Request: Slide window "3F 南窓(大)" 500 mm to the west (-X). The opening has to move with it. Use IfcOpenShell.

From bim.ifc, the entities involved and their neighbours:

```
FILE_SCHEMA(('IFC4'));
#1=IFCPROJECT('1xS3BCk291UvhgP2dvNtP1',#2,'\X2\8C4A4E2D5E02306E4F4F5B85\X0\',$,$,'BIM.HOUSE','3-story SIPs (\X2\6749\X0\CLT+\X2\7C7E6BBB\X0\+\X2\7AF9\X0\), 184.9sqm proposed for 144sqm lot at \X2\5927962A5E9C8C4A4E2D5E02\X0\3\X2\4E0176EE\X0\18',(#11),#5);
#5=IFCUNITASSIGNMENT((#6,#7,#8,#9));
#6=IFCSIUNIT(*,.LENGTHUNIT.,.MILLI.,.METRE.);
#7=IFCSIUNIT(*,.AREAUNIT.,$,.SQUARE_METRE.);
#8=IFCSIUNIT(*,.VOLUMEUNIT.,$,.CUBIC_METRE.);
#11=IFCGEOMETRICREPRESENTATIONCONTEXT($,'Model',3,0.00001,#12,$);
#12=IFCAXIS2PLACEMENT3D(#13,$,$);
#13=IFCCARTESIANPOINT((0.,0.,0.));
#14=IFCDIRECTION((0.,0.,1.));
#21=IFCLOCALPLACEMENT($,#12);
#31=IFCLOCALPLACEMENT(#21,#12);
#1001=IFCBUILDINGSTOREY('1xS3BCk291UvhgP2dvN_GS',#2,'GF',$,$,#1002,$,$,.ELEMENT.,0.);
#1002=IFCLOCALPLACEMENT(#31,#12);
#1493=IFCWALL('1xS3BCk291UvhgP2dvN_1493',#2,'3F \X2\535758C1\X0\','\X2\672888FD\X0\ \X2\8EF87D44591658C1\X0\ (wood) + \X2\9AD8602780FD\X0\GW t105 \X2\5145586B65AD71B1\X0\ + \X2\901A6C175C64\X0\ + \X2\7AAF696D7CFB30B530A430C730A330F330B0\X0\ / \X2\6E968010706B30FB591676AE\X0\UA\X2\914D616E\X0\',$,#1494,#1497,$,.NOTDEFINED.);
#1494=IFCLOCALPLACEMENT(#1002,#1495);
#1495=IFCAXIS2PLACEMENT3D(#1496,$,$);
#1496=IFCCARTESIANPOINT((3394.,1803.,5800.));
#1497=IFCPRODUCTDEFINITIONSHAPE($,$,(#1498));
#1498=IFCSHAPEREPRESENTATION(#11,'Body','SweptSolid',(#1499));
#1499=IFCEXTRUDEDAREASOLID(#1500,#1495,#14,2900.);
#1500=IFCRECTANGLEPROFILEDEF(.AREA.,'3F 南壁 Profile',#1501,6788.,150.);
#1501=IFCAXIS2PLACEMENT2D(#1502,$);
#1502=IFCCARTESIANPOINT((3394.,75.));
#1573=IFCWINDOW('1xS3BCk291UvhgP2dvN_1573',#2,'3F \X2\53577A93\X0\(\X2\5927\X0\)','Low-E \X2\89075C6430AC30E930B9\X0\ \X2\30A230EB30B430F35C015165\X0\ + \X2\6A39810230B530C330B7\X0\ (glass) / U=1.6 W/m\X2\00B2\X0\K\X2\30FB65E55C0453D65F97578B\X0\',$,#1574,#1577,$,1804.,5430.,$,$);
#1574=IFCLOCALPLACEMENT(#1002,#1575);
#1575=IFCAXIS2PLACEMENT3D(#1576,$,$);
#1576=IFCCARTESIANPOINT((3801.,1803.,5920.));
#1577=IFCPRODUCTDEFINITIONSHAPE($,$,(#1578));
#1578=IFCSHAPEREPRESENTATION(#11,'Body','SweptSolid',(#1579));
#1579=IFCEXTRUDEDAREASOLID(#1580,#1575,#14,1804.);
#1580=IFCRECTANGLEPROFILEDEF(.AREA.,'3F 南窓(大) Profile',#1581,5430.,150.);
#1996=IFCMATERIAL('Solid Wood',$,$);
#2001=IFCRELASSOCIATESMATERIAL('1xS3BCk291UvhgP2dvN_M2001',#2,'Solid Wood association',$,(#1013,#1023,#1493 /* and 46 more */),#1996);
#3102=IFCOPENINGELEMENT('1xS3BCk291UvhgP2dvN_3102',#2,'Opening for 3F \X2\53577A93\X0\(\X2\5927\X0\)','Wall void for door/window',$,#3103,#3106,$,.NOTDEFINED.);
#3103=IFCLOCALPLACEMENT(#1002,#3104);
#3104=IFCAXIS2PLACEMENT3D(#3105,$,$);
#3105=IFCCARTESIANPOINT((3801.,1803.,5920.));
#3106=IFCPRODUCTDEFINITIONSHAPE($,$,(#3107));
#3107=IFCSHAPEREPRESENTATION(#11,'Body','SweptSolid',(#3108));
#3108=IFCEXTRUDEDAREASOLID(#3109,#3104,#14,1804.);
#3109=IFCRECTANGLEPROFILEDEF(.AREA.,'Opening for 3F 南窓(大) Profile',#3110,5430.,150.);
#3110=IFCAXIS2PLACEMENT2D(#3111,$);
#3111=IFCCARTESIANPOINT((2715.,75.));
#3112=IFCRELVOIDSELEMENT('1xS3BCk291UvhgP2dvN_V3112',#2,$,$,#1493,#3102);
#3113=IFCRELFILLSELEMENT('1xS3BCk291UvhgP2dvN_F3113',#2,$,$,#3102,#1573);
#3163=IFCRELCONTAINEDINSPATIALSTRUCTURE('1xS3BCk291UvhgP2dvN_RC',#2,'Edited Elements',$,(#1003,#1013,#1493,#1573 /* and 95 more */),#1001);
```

```python
import ifcopenshell
import ifcopenshell.api.geometry
import ifcopenshell.util.placement
import ifcopenshell.util.unit

model = ifcopenshell.open("bim.ifc")
unit_scale = ifcopenshell.util.unit.calculate_unit_scale(model)

window = model.by_guid("1xS3BCk291UvhgP2dvN_1573")
opening = window.FillsVoids[0].RelatingOpeningElement
wall = opening.VoidsElements[0].RelatingBuildingElement

wall_matrix = ifcopenshell.util.placement.get_local_placement(wall.ObjectPlacement)
shift = wall_matrix[:3, 0] * -0.5 / unit_scale
before = ifcopenshell.util.placement.get_local_placement(window.ObjectPlacement)[:3, 3].copy()

# The window is not placed relative to its opening, so move both.
for product in (opening, window):
    matrix = ifcopenshell.util.placement.get_local_placement(product.ObjectPlacement)
    matrix[:3, 3] += shift
    ifcopenshell.api.geometry.edit_object_placement(model, product=product, matrix=matrix, is_si=False)

after = ifcopenshell.util.placement.get_local_placement(window.ObjectPlacement)[:3, 3]
print("window moved by", (after - before).round(3) + 0.0)

model.write("bim_v2.ifc")
```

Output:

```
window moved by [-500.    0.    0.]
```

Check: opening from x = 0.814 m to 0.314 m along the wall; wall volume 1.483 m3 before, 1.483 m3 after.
